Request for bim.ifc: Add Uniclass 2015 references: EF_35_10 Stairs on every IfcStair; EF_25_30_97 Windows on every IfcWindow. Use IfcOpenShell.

First a look at what the model holds.

```python
import ifcopenshell

model = ifcopenshell.open("bim.ifc")
print(model.schema)
print("classifications:", [c.Name for c in model.by_type("IfcClassification")])
for ifc_class in ("IfcDoor", "IfcRoof", "IfcStair", "IfcWall", "IfcWindow"):
    print(ifc_class, len(model.by_type(ifc_class)))
```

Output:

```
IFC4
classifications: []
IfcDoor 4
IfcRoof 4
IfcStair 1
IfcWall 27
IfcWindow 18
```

```python
import ifcopenshell
import ifcopenshell.api.classification

model = ifcopenshell.open("bim.ifc")

system = ifcopenshell.api.classification.add_classification(model, classification="Uniclass 2015")

codes = {
    "IfcStair": ("EF_35_10", "Stairs"),
    "IfcWindow": ("EF_25_30_97", "Windows"),
}
for ifc_class, (code, name) in codes.items():
    products = model.by_type(ifc_class)
    ifcopenshell.api.classification.add_reference(
        model, products=products, classification=system, identification=code, name=name
    )
    print(code, len(products))

model.write("bim-out.ifc")
```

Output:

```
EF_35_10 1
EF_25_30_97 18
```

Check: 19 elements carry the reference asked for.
